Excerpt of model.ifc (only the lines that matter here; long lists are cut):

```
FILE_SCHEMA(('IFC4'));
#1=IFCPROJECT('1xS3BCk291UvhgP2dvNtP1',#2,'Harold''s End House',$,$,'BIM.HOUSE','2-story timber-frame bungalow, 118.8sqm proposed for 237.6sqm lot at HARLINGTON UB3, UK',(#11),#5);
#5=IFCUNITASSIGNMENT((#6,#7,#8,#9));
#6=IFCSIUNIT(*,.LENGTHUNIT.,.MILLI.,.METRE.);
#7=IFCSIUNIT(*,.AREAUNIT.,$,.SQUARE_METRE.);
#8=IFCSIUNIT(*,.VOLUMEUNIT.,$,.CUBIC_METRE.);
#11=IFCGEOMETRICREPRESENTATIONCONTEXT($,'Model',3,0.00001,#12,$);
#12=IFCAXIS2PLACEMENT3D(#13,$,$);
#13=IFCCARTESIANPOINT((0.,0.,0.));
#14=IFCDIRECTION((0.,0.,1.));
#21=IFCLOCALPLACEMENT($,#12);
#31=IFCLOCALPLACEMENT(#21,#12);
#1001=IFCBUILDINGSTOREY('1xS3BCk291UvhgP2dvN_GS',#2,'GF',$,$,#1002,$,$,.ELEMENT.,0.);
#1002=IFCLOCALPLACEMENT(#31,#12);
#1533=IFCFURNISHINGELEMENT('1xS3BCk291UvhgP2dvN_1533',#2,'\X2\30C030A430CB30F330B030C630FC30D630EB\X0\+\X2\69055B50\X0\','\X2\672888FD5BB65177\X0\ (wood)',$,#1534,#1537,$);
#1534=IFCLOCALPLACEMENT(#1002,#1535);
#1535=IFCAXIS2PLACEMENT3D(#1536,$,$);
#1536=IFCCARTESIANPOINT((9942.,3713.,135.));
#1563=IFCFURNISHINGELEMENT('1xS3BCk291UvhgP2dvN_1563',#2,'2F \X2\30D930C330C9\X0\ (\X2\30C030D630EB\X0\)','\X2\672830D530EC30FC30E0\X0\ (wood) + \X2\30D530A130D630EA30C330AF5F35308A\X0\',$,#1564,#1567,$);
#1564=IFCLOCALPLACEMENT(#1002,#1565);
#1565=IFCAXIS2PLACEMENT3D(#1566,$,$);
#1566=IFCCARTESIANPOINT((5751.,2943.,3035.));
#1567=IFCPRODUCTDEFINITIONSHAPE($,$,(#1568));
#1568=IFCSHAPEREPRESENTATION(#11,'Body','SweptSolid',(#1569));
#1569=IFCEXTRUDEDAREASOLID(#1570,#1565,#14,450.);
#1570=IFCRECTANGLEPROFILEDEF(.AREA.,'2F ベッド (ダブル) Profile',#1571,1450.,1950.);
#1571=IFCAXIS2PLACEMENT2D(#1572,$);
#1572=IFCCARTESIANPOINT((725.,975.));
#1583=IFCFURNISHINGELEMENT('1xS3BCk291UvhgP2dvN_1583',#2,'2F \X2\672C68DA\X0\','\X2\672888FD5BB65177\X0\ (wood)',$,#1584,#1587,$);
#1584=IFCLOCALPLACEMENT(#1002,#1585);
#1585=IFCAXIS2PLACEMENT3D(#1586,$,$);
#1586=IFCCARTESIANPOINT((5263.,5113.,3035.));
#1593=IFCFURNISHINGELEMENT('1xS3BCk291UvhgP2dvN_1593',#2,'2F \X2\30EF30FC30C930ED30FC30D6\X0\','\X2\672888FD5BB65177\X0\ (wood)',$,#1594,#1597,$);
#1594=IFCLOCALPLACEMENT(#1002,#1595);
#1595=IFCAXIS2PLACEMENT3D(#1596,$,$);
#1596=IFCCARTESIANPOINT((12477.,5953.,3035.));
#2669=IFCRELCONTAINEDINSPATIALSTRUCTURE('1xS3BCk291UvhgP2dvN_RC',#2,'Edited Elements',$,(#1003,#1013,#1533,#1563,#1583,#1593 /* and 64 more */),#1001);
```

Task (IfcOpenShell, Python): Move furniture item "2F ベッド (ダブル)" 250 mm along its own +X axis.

```python
import ifcopenshell
import ifcopenshell.api.geometry
import ifcopenshell.util.placement
import ifcopenshell.util.unit

model = ifcopenshell.open("model.ifc")
unit_scale = ifcopenshell.util.unit.calculate_unit_scale(model)

item = model.by_guid("1xS3BCk291UvhgP2dvN_1563")
matrix = ifcopenshell.util.placement.get_local_placement(item.ObjectPlacement)
matrix[:3, 3] += matrix[:3, 0] * 0.25 / unit_scale
ifcopenshell.api.geometry.edit_object_placement(model, product=item, matrix=matrix, is_si=False)

print(ifcopenshell.util.placement.get_local_placement(item.ObjectPlacement).round(3) + 0.0)

model.write("model_rev.ifc")
```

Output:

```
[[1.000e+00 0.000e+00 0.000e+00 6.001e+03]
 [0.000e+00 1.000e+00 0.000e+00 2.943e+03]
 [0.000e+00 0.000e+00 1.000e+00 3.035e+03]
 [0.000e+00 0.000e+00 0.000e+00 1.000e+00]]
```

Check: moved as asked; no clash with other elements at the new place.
